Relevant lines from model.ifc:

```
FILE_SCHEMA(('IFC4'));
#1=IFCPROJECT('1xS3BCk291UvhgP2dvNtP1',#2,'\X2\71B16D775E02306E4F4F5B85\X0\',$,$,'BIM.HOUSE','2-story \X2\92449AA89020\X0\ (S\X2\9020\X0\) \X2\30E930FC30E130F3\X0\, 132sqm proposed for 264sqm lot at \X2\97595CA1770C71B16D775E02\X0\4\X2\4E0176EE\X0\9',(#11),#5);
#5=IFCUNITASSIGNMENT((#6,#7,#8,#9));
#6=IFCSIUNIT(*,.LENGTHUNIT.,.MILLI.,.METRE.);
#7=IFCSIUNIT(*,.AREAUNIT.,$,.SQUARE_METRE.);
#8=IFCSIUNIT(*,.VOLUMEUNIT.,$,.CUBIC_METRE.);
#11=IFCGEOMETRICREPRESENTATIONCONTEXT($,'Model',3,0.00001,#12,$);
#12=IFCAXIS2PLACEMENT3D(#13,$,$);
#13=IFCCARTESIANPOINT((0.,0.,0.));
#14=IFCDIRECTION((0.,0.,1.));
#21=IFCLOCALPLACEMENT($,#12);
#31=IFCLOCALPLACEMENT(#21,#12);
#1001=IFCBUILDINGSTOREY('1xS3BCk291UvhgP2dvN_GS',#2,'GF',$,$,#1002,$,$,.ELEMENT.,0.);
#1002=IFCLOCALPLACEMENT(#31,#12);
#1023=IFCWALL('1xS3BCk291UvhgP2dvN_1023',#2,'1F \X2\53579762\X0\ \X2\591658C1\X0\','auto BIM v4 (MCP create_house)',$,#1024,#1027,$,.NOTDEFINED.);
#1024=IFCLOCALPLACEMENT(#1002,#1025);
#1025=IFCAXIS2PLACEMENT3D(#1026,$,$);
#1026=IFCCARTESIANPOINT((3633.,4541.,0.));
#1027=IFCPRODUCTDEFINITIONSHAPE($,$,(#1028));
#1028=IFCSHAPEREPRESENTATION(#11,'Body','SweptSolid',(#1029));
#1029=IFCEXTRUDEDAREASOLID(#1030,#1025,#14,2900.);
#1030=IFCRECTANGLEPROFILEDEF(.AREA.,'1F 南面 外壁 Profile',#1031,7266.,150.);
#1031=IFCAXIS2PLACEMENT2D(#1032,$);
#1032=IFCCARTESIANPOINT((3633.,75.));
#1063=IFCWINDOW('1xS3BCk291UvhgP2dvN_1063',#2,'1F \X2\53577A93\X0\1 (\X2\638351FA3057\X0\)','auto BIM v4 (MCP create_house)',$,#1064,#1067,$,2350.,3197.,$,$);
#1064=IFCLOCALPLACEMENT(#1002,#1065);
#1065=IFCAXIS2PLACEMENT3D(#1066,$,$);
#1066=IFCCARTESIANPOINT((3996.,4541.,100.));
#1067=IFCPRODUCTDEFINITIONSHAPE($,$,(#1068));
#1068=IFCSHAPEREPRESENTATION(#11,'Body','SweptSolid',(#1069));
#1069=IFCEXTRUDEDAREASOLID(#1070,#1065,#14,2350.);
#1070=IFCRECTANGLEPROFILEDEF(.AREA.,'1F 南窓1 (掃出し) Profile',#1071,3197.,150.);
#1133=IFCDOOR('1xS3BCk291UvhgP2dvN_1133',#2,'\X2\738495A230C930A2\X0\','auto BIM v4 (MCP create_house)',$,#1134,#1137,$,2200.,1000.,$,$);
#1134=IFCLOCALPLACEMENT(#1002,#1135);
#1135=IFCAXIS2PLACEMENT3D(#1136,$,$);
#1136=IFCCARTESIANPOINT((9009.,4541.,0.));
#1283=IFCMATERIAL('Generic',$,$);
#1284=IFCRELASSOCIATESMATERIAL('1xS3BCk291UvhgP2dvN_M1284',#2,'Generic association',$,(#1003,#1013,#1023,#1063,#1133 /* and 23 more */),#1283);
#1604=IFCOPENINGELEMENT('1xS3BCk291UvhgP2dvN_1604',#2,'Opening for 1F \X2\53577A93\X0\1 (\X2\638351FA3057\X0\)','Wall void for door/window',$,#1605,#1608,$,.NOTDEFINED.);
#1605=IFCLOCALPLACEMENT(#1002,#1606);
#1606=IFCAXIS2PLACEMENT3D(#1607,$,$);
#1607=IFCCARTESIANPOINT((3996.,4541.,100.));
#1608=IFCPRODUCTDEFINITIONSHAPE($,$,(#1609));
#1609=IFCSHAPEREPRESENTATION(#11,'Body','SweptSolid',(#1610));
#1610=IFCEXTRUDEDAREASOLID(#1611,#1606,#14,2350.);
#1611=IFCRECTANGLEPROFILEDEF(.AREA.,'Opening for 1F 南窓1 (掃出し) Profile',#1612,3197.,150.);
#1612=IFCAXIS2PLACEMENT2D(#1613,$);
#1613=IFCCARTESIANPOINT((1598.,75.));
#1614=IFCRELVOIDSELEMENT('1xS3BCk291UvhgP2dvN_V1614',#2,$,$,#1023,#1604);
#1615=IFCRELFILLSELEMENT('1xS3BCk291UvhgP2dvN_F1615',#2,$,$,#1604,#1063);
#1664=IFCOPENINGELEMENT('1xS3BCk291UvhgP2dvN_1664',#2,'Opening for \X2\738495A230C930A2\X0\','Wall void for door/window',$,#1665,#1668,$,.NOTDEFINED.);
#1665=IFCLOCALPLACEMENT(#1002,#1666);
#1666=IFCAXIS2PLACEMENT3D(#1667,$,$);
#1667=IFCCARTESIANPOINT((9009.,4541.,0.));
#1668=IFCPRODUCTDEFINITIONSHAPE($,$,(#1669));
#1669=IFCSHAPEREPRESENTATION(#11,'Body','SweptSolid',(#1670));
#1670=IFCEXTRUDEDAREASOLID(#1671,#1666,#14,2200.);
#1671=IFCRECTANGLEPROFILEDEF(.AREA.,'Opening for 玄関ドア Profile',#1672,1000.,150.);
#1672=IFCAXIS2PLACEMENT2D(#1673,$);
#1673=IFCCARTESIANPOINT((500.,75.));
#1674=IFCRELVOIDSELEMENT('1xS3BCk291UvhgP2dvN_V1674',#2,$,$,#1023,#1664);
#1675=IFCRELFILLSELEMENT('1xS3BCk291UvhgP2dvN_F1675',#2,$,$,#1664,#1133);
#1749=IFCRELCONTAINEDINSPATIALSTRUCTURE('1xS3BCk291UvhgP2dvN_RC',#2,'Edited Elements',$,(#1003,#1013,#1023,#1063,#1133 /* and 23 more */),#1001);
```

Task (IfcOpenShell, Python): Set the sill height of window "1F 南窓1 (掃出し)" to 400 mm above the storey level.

```python
import numpy as np
import ifcopenshell
import ifcopenshell.api.geometry
import ifcopenshell.geom
import ifcopenshell.util.element
import ifcopenshell.util.placement
import ifcopenshell.util.shape
import ifcopenshell.util.unit

model = ifcopenshell.open("model.ifc")
unit_scale = ifcopenshell.util.unit.calculate_unit_scale(model)

window = model.by_guid("1xS3BCk291UvhgP2dvN_1063")
opening = window.FillsVoids[0].RelatingOpeningElement
storey = ifcopenshell.util.element.get_container(window, ifc_class="IfcBuildingStorey")
level = ifcopenshell.util.placement.get_local_placement(storey.ObjectPlacement)[2, 3]

# The opening's origin need not be at the sill, so measure its lowest point.
shape = ifcopenshell.geom.create_shape(ifcopenshell.geom.settings(), opening)
bottom = ifcopenshell.util.shape.get_shape_bottom_elevation(shape, shape.geometry) / unit_scale
dz = level + 0.4 / unit_scale - bottom

shift = np.array([0.0, 0.0, dz])
# The window is not placed relative to its opening, so move both.
for product in (opening, window):
    matrix = ifcopenshell.util.placement.get_local_placement(product.ObjectPlacement)
    matrix[:3, 3] += shift
    ifcopenshell.api.geometry.edit_object_placement(model, product=product, matrix=matrix, is_si=False)

print(f"moved by {dz * unit_scale:+.3f} m")

model.write("model_rev.ifc")
```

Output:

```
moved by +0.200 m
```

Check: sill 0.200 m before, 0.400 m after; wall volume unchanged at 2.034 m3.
